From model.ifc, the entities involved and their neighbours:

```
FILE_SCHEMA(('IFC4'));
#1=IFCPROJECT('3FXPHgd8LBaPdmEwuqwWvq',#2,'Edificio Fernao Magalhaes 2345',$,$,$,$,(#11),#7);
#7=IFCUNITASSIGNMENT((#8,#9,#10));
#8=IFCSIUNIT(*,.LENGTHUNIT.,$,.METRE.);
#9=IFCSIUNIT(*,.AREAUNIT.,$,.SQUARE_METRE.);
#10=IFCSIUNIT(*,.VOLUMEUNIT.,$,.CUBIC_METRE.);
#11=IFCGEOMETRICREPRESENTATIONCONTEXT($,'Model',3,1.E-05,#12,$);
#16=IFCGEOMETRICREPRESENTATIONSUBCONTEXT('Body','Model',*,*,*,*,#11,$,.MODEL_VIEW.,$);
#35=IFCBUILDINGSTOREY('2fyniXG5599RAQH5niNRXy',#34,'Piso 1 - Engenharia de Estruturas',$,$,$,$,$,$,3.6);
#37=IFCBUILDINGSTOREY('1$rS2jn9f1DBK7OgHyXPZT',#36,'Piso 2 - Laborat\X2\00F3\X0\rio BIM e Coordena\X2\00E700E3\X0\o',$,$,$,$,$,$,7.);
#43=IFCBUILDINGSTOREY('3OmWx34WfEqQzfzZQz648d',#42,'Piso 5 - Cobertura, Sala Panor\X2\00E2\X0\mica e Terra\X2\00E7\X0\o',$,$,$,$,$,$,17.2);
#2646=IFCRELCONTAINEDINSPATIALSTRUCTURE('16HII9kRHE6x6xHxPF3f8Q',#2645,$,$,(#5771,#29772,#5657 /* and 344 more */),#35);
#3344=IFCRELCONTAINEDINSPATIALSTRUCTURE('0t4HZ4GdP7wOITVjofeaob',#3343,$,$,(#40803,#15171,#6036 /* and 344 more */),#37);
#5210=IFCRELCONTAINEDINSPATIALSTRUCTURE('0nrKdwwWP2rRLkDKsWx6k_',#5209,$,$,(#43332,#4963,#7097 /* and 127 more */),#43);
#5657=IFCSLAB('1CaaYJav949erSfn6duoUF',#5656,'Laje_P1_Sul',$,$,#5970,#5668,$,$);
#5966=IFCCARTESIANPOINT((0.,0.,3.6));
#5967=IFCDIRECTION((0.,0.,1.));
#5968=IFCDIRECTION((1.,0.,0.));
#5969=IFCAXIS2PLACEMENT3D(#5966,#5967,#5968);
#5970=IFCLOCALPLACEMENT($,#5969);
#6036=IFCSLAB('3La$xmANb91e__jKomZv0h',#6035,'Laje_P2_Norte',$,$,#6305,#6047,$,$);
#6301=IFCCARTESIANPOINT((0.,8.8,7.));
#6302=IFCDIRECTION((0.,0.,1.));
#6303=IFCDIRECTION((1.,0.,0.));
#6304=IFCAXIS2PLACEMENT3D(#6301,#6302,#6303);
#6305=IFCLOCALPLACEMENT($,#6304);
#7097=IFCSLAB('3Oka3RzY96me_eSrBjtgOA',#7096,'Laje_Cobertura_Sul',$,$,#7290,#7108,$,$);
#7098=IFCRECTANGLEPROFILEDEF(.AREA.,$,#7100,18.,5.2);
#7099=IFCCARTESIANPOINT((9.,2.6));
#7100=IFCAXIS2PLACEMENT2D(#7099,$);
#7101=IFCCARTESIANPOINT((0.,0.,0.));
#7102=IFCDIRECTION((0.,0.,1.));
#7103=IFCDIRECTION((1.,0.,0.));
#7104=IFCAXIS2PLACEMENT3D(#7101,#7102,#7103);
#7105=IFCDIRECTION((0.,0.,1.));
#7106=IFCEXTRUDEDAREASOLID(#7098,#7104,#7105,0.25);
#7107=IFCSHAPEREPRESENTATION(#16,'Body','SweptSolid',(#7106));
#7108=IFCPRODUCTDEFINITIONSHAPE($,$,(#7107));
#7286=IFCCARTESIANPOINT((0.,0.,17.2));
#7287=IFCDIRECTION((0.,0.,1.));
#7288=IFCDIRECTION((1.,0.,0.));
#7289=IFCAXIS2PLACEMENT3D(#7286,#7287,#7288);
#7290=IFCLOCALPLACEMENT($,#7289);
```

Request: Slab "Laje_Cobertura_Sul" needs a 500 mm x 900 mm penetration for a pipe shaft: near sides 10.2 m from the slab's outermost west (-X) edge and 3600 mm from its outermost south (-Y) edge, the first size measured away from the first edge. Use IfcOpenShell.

```python
import numpy as np
import ifcopenshell
import ifcopenshell.api.feature
import ifcopenshell.api.geometry
import ifcopenshell.api.root
import ifcopenshell.geom
import ifcopenshell.util.placement
import ifcopenshell.util.representation
import ifcopenshell.util.shape
import ifcopenshell.util.unit

model = ifcopenshell.open("model.ifc")
unit_scale = ifcopenshell.util.unit.calculate_unit_scale(model)
settings = ifcopenshell.geom.settings()


def volume(element):
    """Net volume in cubic metres, openings subtracted."""
    shape = ifcopenshell.geom.create_shape(settings, element)
    return ifcopenshell.util.shape.get_volume(shape.geometry)


slab = model.by_guid("3Oka3RzY96me_eSrBjtgOA")
before = volume(slab)

# Extent in the slab's own axes, in metres. The edges named are its -X and -Y sides.
slab_shape = ifcopenshell.geom.create_shape(settings, slab)
vertices = ifcopenshell.util.shape.get_vertices(slab_shape.geometry)
x_min, y_min, bottom = vertices.min(axis=0)
top = vertices[:, 2].max()

opening = ifcopenshell.api.root.create_entity(model, ifc_class="IfcOpeningElement", name="Pipe shaft opening", predefined_type="OPENING")
context = ifcopenshell.util.representation.get_context(model, "Model", "Body", "MODEL_VIEW")
width, depth = 0.5, 0.9
outline = [(0.0, 0.0), (width, 0.0), (width, depth), (0.0, depth), (0.0, 0.0)]
# Overshoot both faces by 50 mm so the cut is clean.
shape = ifcopenshell.api.geometry.add_slab_representation(
    model, context=context, depth=top - bottom + 0.1, polyline=outline
)
ifcopenshell.api.geometry.assign_representation(model, product=opening, representation=shape)

matrix = ifcopenshell.util.placement.get_local_placement(slab.ObjectPlacement)
matrix[:, 3] = matrix @ np.append(np.array([x_min + 10.2, y_min + 3.6, bottom - 0.05]) / unit_scale, 1.0)
ifcopenshell.api.geometry.edit_object_placement(model, product=opening, matrix=matrix, is_si=False)
ifcopenshell.api.feature.add_feature(model, feature=opening, element=slab)

after = volume(slab)

print(f"slab volume {before:.3f} -> {after:.3f} m3")

model.write("model-out.ifc")
```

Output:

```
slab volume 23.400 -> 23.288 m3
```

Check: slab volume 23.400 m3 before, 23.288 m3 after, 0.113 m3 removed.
